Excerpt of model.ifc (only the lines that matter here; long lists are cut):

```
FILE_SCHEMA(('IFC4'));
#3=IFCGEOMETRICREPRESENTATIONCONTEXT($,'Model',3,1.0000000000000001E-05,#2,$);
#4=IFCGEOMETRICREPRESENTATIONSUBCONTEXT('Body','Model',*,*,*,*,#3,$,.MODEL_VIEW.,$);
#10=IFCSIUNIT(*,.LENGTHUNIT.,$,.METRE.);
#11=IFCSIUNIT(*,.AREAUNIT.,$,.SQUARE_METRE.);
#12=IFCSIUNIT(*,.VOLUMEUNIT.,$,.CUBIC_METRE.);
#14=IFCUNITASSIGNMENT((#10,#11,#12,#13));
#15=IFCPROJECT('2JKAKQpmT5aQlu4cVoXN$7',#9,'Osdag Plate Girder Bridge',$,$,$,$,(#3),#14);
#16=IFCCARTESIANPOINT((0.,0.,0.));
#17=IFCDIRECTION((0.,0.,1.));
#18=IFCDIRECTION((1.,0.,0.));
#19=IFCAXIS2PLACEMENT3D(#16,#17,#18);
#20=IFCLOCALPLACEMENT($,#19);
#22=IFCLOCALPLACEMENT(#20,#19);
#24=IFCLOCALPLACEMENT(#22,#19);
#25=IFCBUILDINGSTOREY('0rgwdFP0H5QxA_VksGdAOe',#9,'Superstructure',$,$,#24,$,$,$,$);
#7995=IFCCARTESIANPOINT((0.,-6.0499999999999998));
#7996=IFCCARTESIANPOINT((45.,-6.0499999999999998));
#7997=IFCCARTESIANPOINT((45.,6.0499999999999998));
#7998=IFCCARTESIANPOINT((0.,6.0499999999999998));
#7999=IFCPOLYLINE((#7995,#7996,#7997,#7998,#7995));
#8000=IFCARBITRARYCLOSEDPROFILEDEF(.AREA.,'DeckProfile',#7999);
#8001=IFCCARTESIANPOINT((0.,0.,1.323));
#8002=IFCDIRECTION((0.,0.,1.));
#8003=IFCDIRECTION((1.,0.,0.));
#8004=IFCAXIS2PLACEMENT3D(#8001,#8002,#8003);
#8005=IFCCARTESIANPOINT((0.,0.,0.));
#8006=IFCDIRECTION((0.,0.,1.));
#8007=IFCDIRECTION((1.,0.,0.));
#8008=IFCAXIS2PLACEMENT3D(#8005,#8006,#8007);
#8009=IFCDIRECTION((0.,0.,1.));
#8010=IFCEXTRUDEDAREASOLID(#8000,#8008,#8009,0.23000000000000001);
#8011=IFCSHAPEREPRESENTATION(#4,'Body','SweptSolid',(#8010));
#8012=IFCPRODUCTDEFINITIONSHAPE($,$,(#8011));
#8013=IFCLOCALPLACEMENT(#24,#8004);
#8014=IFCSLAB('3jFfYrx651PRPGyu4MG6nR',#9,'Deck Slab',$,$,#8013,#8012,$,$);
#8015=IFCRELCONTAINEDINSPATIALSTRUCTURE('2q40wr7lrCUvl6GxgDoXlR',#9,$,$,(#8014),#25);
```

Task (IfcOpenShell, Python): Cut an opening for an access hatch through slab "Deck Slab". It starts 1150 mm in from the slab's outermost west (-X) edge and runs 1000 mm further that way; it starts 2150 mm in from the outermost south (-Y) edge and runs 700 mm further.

```python
import numpy as np
import ifcopenshell
import ifcopenshell.api.feature
import ifcopenshell.api.geometry
import ifcopenshell.api.root
import ifcopenshell.geom
import ifcopenshell.util.placement
import ifcopenshell.util.representation
import ifcopenshell.util.shape
import ifcopenshell.util.unit

model = ifcopenshell.open("model.ifc")
unit_scale = ifcopenshell.util.unit.calculate_unit_scale(model)
settings = ifcopenshell.geom.settings()


def volume(element):
    """Net volume in cubic metres, openings subtracted."""
    shape = ifcopenshell.geom.create_shape(settings, element)
    return ifcopenshell.util.shape.get_volume(shape.geometry)


slab = model.by_guid("3jFfYrx651PRPGyu4MG6nR")
before = volume(slab)

# Extent in the slab's own axes, in metres. The edges named are its -X and -Y sides.
slab_shape = ifcopenshell.geom.create_shape(settings, slab)
vertices = ifcopenshell.util.shape.get_vertices(slab_shape.geometry)
x_min, y_min, bottom = vertices.min(axis=0)
top = vertices[:, 2].max()

opening = ifcopenshell.api.root.create_entity(model, ifc_class="IfcOpeningElement", name="Access hatch opening", predefined_type="OPENING")
context = ifcopenshell.util.representation.get_context(model, "Model", "Body", "MODEL_VIEW")
width, depth = 1, 0.7
outline = [(0.0, 0.0), (width, 0.0), (width, depth), (0.0, depth), (0.0, 0.0)]
# Overshoot both faces by 50 mm so the cut is clean.
shape = ifcopenshell.api.geometry.add_slab_representation(
    model, context=context, depth=top - bottom + 0.1, polyline=outline
)
ifcopenshell.api.geometry.assign_representation(model, product=opening, representation=shape)

matrix = ifcopenshell.util.placement.get_local_placement(slab.ObjectPlacement)
matrix[:, 3] = matrix @ np.append(np.array([x_min + 1.15, y_min + 2.15, bottom - 0.05]) / unit_scale, 1.0)
ifcopenshell.api.geometry.edit_object_placement(model, product=opening, matrix=matrix, is_si=False)
ifcopenshell.api.feature.add_feature(model, feature=opening, element=slab)

after = volume(slab)

print(f"slab volume {before:.3f} -> {after:.3f} m3")

model.write("model_updated.ifc")
```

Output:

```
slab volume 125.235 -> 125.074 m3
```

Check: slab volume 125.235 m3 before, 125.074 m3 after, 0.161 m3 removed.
